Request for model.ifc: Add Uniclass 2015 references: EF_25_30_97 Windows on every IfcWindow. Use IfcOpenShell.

First a look at what the model holds.

```python
import ifcopenshell

model = ifcopenshell.open("model.ifc")
print(model.schema)
print("classifications:", [c.Name for c in model.by_type("IfcClassification")])
for ifc_class in ("IfcDoor", "IfcRoof", "IfcStair", "IfcWall", "IfcWindow"):
    print(ifc_class, len(model.by_type(ifc_class)))
```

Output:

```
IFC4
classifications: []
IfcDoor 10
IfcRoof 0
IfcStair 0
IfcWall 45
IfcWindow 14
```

```python
import ifcopenshell
import ifcopenshell.api.classification

model = ifcopenshell.open("model.ifc")

system = ifcopenshell.api.classification.add_classification(model, classification="Uniclass 2015")

codes = {
    "IfcWindow": ("EF_25_30_97", "Windows"),
}
for ifc_class, (code, name) in codes.items():
    products = model.by_type(ifc_class)
    ifcopenshell.api.classification.add_reference(
        model, products=products, classification=system, identification=code, name=name
    )
    print(code, len(products))

model.write("model_updated.ifc")
```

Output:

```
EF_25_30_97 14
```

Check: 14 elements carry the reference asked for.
